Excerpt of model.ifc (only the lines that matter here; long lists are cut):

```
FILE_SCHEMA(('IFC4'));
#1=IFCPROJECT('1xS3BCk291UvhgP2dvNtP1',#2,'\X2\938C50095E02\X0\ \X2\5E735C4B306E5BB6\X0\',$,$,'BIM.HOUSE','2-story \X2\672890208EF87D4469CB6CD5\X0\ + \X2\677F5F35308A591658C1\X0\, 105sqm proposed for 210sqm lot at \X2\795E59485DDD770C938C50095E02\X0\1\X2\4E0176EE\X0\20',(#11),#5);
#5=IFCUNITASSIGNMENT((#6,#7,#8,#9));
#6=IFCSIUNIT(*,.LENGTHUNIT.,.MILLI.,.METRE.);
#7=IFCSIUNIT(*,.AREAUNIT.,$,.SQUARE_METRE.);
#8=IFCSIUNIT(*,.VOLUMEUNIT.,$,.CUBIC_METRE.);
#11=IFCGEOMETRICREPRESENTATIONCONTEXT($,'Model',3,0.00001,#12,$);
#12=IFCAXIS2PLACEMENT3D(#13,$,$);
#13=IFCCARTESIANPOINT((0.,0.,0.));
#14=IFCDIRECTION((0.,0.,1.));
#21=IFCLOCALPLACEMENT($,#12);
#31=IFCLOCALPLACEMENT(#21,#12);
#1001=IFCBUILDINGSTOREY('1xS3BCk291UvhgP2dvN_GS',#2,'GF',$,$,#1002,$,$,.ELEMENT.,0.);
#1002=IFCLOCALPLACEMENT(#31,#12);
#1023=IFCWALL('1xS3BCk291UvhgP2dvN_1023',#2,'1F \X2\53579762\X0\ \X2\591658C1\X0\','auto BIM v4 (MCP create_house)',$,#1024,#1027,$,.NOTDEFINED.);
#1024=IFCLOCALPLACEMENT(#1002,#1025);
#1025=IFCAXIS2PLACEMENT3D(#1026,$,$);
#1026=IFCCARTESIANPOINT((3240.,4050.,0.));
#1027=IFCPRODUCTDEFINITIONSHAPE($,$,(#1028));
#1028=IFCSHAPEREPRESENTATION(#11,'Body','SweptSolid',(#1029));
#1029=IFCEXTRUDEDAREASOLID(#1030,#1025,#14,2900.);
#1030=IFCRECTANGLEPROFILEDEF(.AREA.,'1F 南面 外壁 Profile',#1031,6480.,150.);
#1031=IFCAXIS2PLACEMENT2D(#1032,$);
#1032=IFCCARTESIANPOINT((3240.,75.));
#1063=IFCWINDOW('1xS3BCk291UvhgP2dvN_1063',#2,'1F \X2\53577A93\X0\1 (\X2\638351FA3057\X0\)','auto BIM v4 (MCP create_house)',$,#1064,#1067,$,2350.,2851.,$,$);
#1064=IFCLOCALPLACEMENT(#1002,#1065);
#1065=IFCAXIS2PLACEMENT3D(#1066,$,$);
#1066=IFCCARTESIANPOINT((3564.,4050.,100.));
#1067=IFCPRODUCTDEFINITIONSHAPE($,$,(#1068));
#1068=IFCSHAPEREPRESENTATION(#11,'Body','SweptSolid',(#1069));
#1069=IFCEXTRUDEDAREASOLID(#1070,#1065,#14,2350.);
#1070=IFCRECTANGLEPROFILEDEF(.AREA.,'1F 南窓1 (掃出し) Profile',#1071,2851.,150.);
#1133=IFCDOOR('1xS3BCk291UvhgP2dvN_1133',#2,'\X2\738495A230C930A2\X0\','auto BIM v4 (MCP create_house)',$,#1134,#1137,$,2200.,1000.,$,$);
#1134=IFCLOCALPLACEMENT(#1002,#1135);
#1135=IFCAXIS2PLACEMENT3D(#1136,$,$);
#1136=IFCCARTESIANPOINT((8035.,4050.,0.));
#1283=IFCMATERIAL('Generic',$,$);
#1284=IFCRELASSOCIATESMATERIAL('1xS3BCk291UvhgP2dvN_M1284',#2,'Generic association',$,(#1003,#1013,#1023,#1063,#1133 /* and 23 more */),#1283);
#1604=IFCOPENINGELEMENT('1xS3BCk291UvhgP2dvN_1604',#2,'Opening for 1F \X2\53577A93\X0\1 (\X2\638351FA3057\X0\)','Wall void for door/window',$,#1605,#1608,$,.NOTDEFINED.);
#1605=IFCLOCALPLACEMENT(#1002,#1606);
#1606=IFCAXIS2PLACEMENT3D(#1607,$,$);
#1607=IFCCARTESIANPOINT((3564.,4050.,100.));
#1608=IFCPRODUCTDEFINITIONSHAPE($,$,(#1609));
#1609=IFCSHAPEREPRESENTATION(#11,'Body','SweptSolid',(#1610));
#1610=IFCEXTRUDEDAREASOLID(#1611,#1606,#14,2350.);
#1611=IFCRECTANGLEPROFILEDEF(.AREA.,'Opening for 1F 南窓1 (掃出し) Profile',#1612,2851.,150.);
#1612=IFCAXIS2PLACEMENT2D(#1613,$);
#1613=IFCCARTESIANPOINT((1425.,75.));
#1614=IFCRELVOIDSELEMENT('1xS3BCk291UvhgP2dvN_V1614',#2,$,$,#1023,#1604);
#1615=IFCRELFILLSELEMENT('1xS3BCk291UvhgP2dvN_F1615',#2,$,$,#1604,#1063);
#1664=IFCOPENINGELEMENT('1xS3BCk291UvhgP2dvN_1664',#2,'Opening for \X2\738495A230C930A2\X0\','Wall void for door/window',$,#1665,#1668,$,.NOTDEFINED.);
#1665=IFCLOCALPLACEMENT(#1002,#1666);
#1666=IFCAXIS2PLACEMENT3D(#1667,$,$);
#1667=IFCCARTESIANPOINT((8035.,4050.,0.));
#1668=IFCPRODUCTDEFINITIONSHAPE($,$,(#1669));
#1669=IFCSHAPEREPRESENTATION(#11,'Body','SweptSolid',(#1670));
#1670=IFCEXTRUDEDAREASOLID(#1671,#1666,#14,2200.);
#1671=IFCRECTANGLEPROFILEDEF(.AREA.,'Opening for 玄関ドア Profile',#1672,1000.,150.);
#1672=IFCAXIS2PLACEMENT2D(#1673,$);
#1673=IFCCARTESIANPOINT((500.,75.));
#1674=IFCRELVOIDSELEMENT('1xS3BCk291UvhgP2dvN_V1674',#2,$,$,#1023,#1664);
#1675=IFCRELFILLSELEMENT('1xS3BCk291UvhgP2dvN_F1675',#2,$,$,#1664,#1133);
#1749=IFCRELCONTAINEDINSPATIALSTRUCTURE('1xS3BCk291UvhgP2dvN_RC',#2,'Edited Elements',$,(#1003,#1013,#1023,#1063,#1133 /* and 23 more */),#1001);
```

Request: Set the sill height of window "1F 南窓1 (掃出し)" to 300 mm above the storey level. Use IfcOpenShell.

```python
import numpy as np
import ifcopenshell
import ifcopenshell.api.geometry
import ifcopenshell.geom
import ifcopenshell.util.element
import ifcopenshell.util.placement
import ifcopenshell.util.shape
import ifcopenshell.util.unit

model = ifcopenshell.open("model.ifc")
unit_scale = ifcopenshell.util.unit.calculate_unit_scale(model)

window = model.by_guid("1xS3BCk291UvhgP2dvN_1063")
opening = window.FillsVoids[0].RelatingOpeningElement
storey = ifcopenshell.util.element.get_container(window, ifc_class="IfcBuildingStorey")
level = ifcopenshell.util.placement.get_local_placement(storey.ObjectPlacement)[2, 3]

# The opening's origin need not be at the sill, so measure its lowest point.
shape = ifcopenshell.geom.create_shape(ifcopenshell.geom.settings(), opening)
bottom = ifcopenshell.util.shape.get_shape_bottom_elevation(shape, shape.geometry) / unit_scale
dz = level + 300.0 - bottom

shift = np.array([0.0, 0.0, dz])
# The window is not placed relative to its opening, so move both.
for product in (opening, window):
    matrix = ifcopenshell.util.placement.get_local_placement(product.ObjectPlacement)
    matrix[:3, 3] += shift
    ifcopenshell.api.geometry.edit_object_placement(model, product=product, matrix=matrix, is_si=False)

print(f"moved by {dz * unit_scale:+.3f} m")

model.write("model_edited.ifc")
```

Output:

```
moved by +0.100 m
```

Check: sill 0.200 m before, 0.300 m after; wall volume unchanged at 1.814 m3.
